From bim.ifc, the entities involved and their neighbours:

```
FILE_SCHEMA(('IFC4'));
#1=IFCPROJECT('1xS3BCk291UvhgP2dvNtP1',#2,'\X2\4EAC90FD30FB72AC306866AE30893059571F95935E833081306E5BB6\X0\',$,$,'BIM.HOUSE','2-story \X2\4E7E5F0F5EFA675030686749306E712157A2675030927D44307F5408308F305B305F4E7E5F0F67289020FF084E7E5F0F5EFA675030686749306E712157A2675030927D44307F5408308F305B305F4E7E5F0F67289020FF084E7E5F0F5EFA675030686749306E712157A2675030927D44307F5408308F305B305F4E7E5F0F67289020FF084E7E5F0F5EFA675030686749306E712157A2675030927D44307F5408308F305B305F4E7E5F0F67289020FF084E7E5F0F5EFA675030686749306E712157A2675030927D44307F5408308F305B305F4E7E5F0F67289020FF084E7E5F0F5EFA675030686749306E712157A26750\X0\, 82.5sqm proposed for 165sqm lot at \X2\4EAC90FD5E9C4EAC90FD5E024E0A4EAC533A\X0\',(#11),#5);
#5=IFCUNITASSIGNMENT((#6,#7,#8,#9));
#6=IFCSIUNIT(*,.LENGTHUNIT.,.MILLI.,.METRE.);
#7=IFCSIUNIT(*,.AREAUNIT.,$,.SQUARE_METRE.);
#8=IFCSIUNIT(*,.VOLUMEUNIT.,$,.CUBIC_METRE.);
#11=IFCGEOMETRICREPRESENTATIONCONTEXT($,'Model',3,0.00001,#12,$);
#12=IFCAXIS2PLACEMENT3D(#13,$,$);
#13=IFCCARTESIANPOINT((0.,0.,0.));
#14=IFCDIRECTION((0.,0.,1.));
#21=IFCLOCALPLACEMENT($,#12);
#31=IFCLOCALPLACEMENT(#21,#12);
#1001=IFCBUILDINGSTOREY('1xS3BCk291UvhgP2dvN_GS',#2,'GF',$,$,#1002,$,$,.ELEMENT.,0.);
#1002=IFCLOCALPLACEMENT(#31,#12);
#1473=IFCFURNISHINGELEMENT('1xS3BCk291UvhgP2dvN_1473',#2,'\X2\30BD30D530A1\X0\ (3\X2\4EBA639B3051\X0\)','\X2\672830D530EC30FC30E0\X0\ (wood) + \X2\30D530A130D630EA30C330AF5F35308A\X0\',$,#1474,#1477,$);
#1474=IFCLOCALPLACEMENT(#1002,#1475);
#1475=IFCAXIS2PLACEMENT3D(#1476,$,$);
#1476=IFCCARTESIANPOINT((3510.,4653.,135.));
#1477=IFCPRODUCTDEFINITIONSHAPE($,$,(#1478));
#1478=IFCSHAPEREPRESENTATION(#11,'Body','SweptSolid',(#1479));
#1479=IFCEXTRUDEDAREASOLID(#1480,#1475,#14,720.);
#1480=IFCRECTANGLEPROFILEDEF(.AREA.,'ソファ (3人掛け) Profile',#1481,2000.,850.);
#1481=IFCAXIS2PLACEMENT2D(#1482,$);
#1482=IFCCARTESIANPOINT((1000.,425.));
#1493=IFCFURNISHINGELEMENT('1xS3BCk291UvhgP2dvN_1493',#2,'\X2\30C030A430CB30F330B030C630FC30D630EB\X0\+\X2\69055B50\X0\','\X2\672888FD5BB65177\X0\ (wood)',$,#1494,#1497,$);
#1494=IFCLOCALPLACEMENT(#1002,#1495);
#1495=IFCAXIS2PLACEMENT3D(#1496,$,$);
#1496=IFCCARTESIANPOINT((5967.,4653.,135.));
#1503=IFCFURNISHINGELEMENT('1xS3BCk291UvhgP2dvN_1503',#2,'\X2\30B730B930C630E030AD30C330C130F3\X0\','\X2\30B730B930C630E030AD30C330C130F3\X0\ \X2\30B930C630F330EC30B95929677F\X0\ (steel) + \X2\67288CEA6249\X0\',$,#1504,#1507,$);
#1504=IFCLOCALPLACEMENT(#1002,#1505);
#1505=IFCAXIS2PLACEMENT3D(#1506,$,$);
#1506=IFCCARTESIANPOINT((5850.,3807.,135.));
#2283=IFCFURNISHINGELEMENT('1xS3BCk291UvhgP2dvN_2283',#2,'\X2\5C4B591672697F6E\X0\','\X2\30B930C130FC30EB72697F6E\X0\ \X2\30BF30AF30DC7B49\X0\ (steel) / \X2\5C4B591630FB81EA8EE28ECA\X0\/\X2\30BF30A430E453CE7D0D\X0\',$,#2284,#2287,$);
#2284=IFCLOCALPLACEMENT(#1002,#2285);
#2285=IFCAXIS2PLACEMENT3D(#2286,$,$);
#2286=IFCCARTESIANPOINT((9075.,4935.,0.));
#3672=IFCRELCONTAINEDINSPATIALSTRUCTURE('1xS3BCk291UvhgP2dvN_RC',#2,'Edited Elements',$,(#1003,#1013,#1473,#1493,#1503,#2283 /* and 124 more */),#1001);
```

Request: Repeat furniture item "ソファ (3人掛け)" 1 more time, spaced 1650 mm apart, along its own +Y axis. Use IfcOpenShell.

```python
import ifcopenshell
import ifcopenshell.api.geometry
import ifcopenshell.api.root
import ifcopenshell.util.element
import ifcopenshell.util.placement
import ifcopenshell.util.unit

model = ifcopenshell.open("bim.ifc")
unit_scale = ifcopenshell.util.unit.calculate_unit_scale(model)


def reuse_history(source, copy):
    """copy_class also copies each property set's owner history, people and application; keep the originals."""
    for rel in copy.IsDefinedBy:
        if rel.is_a("IfcRelDefinesByProperties") and (history := rel.RelatingPropertyDefinition.OwnerHistory):
            rel.RelatingPropertyDefinition.OwnerHistory = source.OwnerHistory
            ifcopenshell.util.element.remove_deep2(model, history)


source = model.by_guid("1xS3BCk291UvhgP2dvN_1473")
base = ifcopenshell.util.placement.get_local_placement(source.ObjectPlacement)
step = base[:3, 1] * 1.65 / unit_scale

for i in range(1, 2):
    copy = ifcopenshell.api.root.copy_class(model, product=source)
    copy.Representation = ifcopenshell.util.element.copy_deep(
        model, source.Representation, exclude=["IfcGeometricRepresentationContext", "IfcRepresentationMap"]
    )
    reuse_history(source, copy)
    matrix = base.copy()
    matrix[:3, 3] += i * step
    print("added at", matrix[:3, 3].round(3) + 0.0)
    ifcopenshell.api.geometry.edit_object_placement(model, product=copy, matrix=matrix, is_si=False)

model.write("bim-out.ifc")
```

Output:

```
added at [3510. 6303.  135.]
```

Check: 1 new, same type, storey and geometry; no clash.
